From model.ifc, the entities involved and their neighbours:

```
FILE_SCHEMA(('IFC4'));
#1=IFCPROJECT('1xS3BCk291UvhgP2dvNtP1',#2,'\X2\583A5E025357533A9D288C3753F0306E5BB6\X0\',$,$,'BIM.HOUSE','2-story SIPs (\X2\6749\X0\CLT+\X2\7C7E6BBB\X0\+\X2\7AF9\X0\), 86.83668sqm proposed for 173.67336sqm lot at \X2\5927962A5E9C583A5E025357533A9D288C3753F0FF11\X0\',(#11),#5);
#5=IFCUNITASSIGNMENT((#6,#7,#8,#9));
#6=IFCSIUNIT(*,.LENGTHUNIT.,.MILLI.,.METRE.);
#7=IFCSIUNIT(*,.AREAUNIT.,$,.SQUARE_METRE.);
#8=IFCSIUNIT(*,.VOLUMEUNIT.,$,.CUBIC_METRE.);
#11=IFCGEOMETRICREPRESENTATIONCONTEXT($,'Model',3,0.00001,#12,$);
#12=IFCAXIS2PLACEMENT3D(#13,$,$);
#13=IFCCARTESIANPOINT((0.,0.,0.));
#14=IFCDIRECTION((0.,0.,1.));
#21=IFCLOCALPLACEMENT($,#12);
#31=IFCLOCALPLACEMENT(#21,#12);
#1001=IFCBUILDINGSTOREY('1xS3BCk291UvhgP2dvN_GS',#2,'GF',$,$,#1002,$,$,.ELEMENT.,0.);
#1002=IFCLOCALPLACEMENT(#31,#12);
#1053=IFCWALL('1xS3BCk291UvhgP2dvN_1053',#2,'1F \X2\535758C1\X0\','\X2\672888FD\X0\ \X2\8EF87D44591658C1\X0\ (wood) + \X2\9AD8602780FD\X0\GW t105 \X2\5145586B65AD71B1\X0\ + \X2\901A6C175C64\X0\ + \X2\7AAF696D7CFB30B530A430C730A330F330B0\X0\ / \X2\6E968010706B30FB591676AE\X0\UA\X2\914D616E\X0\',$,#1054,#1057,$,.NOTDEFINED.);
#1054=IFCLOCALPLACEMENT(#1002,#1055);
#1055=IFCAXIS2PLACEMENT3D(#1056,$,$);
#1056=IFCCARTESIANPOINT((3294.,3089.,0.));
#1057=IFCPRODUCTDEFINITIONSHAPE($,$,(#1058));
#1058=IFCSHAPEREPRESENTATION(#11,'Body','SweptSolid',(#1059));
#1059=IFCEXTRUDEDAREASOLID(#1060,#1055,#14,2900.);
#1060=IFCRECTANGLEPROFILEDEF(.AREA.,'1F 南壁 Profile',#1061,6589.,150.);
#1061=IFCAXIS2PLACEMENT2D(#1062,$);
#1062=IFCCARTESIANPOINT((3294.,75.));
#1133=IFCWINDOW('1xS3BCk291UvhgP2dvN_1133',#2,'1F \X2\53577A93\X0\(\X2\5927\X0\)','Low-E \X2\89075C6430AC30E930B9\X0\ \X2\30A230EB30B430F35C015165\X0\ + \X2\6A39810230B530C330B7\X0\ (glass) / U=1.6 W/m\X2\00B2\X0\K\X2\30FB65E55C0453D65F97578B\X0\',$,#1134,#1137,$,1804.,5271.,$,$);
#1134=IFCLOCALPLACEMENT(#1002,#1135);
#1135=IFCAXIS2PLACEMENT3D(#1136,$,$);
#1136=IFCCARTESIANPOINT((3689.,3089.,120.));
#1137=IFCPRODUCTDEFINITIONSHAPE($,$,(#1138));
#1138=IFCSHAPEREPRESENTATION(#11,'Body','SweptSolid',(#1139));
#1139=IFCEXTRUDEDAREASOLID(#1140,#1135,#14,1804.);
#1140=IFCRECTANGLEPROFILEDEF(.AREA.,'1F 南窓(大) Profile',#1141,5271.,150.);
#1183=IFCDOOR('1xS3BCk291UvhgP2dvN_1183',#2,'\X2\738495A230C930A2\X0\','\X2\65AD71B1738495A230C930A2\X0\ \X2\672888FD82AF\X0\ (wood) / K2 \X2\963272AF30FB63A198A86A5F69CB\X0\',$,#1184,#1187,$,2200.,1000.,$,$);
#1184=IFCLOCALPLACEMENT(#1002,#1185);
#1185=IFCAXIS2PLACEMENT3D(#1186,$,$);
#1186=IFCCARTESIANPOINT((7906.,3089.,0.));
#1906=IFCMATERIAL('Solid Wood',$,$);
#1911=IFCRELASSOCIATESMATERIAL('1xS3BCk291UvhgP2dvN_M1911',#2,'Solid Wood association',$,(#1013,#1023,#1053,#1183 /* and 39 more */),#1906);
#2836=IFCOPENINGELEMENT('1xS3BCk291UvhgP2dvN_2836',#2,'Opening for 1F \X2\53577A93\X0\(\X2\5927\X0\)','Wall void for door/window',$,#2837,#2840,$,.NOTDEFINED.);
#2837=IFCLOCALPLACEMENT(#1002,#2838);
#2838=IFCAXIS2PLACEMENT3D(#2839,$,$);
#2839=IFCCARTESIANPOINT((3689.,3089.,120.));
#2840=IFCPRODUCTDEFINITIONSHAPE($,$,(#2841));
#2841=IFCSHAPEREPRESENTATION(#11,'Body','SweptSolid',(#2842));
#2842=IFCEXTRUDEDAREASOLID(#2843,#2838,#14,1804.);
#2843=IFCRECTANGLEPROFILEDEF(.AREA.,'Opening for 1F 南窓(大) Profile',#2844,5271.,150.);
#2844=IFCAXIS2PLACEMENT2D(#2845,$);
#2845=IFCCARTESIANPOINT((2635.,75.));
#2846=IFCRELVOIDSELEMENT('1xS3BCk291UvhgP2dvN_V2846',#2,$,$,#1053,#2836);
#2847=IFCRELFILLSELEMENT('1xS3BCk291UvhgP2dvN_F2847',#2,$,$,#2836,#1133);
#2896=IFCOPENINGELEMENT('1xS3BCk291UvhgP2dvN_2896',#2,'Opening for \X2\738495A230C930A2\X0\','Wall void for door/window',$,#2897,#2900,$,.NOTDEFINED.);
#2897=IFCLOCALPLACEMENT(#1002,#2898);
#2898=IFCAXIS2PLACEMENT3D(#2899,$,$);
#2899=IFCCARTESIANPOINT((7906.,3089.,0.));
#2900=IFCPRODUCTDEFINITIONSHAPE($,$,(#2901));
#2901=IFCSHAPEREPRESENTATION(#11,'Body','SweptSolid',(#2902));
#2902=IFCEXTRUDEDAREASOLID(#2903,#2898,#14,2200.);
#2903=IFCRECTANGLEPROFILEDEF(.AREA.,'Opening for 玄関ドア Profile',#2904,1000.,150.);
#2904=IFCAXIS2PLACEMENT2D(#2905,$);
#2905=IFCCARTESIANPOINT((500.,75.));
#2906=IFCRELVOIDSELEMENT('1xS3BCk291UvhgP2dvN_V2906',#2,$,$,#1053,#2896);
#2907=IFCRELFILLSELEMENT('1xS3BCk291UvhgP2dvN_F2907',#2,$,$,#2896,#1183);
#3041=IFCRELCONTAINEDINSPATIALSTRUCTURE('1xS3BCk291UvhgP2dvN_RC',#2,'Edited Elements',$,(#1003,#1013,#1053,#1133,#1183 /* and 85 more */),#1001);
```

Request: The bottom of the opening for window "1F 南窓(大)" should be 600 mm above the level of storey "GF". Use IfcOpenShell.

```python
import numpy as np
import ifcopenshell
import ifcopenshell.api.geometry
import ifcopenshell.geom
import ifcopenshell.util.element
import ifcopenshell.util.placement
import ifcopenshell.util.shape
import ifcopenshell.util.unit

model = ifcopenshell.open("model.ifc")
unit_scale = ifcopenshell.util.unit.calculate_unit_scale(model)

window = model.by_id(1133)
opening = window.FillsVoids[0].RelatingOpeningElement
storey = ifcopenshell.util.element.get_container(window, ifc_class="IfcBuildingStorey")
level = ifcopenshell.util.placement.get_local_placement(storey.ObjectPlacement)[2, 3]

# The opening's origin need not be at the sill, so measure its lowest point.
shape = ifcopenshell.geom.create_shape(ifcopenshell.geom.settings(), opening)
bottom = ifcopenshell.util.shape.get_shape_bottom_elevation(shape, shape.geometry) / unit_scale
dz = level + 0.6 / unit_scale - bottom

shift = np.array([0.0, 0.0, dz])
# The window is not placed relative to its opening, so move both.
for product in (opening, window):
    matrix = ifcopenshell.util.placement.get_local_placement(product.ObjectPlacement)
    matrix[:3, 3] += shift
    ifcopenshell.api.geometry.edit_object_placement(model, product=product, matrix=matrix, is_si=False)

print(f"moved by {dz * unit_scale:+.3f} m")

model.write("model_edited.ifc")
```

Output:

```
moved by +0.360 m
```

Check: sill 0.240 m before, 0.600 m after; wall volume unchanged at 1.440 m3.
